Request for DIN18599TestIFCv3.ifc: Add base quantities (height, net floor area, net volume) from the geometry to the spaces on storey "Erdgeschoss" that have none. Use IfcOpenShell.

First a look at what the model holds.

```python
import ifcopenshell
import ifcopenshell.util.element
import ifcopenshell.util.unit

model = ifcopenshell.open("DIN18599TestIFCv3.ifc")
print(model.schema)
for unit_type in ("LENGTHUNIT", "AREAUNIT", "VOLUMEUNIT"):
    print(unit_type, ifcopenshell.util.unit.calculate_unit_scale(model, unit_type))
storey = next(s for s in model.by_type("IfcBuildingStorey") if s.Name == "Erdgeschoss")
spaces = [e for e in ifcopenshell.util.element.get_decomposition(storey) if e.is_a("IfcSpace")]
for e in sorted(spaces, key=lambda e: e.id()):
    print(e.id(), e.is_a(), e.Name, list(ifcopenshell.util.element.get_psets(e, qtos_only=True)), sep=" | ")
```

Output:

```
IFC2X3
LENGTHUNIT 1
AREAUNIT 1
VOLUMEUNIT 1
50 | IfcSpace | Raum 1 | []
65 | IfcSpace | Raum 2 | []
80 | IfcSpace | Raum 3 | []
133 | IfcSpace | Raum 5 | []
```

```python
import ifcopenshell
import ifcopenshell.api.pset
import ifcopenshell.geom
import ifcopenshell.util.element
import ifcopenshell.util.shape
import ifcopenshell.util.unit

model = ifcopenshell.open("DIN18599TestIFCv3.ifc")
unit_scale = ifcopenshell.util.unit.calculate_unit_scale(model)
area_scale = ifcopenshell.util.unit.calculate_unit_scale(model, "AREAUNIT")
volume_scale = ifcopenshell.util.unit.calculate_unit_scale(model, "VOLUMEUNIT")
settings = ifcopenshell.geom.settings()

storey = next(s for s in model.by_type("IfcBuildingStorey") if s.Name == "Erdgeschoss")
spaces = [e for e in ifcopenshell.util.element.get_decomposition(storey) if e.is_a("IfcSpace")]

for e in sorted(spaces, key=lambda e: e.id()):
    if ifcopenshell.util.element.get_psets(e, qtos_only=True, should_inherit=False):
        continue
    # Geometry comes back in metres, in the element's own axes.
    shape = ifcopenshell.geom.create_shape(settings, e)
    values = {
        "Height": ifcopenshell.util.shape.get_z(shape.geometry) / unit_scale,
        "NetFloorArea": ifcopenshell.util.shape.get_footprint_area(shape.geometry) / area_scale,
        "NetVolume": ifcopenshell.util.shape.get_volume(shape.geometry) / volume_scale,
    }
    qto = ifcopenshell.api.pset.add_qto(model, product=e, name="BaseQuantities")
    ifcopenshell.api.pset.edit_qto(model, qto=qto, properties=values)
    print(e.id(), {k: round(v, 3) for k, v in values.items()})

model.write("DIN18599TestIFCv3-out.ifc")
```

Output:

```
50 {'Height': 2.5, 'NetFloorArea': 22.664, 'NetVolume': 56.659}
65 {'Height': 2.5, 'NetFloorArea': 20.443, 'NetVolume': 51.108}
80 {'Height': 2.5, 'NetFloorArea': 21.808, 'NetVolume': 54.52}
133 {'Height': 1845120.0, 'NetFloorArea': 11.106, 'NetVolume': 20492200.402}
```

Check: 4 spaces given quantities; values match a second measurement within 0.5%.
